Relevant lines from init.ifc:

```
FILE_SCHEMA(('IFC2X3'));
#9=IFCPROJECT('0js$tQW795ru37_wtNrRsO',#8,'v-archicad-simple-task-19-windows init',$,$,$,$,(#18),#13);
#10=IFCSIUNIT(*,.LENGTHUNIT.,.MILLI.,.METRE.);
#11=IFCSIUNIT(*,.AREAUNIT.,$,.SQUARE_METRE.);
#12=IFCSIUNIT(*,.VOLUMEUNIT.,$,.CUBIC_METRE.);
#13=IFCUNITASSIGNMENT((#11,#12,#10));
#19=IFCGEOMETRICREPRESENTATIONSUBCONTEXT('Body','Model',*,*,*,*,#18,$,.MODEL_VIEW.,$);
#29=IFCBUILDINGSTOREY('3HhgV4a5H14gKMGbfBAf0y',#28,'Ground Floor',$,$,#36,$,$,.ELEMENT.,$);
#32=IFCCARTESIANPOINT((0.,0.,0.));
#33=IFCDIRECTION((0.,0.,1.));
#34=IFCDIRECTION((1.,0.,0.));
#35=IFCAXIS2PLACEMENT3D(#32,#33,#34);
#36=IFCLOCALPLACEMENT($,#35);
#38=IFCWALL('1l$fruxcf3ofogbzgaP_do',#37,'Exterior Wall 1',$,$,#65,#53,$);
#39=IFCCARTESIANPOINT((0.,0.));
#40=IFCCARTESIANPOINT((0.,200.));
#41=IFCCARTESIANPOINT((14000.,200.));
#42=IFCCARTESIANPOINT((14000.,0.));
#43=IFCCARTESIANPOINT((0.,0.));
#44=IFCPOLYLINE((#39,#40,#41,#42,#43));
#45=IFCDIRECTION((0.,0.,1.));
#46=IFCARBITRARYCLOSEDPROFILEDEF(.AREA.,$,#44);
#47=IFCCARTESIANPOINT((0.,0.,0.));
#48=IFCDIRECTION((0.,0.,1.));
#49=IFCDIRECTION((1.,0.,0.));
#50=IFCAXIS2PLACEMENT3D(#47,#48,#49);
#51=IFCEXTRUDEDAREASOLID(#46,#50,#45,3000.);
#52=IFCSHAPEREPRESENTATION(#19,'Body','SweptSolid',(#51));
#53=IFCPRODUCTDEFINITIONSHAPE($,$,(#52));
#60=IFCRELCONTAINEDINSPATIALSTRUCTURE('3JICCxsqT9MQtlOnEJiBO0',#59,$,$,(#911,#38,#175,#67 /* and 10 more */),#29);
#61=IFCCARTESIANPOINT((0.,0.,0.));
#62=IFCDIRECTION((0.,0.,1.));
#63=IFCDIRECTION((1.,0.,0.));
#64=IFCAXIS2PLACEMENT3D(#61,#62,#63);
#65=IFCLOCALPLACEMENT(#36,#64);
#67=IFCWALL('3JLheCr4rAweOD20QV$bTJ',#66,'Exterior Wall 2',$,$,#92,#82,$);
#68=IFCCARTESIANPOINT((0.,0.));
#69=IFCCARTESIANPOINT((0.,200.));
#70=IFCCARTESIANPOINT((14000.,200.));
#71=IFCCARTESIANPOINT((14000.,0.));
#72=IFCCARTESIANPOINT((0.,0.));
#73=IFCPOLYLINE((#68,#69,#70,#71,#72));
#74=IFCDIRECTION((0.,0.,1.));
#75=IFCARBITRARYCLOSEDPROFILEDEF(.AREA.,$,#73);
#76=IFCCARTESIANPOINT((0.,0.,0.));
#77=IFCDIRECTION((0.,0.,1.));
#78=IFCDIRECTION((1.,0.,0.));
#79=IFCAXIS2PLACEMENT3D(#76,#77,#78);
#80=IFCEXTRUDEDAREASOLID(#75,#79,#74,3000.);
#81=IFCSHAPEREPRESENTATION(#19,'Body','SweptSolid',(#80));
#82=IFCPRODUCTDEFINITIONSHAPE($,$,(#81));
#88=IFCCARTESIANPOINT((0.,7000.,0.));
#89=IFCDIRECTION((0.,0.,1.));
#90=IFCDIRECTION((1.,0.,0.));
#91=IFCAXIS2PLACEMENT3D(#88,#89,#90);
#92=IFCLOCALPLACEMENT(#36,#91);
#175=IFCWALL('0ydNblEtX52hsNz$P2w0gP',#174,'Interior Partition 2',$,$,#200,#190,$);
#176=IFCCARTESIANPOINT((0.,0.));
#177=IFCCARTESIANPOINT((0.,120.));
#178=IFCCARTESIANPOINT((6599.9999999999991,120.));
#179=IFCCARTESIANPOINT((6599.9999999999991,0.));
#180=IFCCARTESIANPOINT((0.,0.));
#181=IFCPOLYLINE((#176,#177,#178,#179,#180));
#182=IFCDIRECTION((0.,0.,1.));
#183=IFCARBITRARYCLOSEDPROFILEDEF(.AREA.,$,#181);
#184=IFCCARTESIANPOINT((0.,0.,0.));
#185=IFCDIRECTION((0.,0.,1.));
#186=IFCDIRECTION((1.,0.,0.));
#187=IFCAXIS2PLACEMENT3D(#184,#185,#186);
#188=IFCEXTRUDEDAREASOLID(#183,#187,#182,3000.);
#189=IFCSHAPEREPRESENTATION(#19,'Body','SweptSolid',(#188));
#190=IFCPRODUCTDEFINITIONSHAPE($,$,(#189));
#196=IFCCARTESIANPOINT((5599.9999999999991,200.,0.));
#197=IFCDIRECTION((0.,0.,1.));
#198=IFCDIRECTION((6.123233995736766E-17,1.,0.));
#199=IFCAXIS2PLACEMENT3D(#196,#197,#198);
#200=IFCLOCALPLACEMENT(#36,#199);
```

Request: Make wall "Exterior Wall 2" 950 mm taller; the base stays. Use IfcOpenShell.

```python
import ifcopenshell
import ifcopenshell.geom
import ifcopenshell.util.representation
import ifcopenshell.util.shape

model = ifcopenshell.open("init.ifc")
settings = ifcopenshell.geom.settings()


def volume(element):
    """Net volume in cubic metres, openings subtracted."""
    shape = ifcopenshell.geom.create_shape(settings, element)
    return ifcopenshell.util.shape.get_volume(shape.geometry)


wall = model.by_guid("3JLheCr4rAweOD20QV$bTJ")
before = volume(wall)

body = ifcopenshell.util.representation.get_representation(wall, "Model", "Body")
solid = body.Items[0]
old_height = solid.Depth
solid.Depth += 950.0
after = volume(wall)

print(f"height {old_height:g} -> {solid.Depth:g}, volume {before:.3f} -> {after:.3f} m3")

model.write("init-out.ifc")
```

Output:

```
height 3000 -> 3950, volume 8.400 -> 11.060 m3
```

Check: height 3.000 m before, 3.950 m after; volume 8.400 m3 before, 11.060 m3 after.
